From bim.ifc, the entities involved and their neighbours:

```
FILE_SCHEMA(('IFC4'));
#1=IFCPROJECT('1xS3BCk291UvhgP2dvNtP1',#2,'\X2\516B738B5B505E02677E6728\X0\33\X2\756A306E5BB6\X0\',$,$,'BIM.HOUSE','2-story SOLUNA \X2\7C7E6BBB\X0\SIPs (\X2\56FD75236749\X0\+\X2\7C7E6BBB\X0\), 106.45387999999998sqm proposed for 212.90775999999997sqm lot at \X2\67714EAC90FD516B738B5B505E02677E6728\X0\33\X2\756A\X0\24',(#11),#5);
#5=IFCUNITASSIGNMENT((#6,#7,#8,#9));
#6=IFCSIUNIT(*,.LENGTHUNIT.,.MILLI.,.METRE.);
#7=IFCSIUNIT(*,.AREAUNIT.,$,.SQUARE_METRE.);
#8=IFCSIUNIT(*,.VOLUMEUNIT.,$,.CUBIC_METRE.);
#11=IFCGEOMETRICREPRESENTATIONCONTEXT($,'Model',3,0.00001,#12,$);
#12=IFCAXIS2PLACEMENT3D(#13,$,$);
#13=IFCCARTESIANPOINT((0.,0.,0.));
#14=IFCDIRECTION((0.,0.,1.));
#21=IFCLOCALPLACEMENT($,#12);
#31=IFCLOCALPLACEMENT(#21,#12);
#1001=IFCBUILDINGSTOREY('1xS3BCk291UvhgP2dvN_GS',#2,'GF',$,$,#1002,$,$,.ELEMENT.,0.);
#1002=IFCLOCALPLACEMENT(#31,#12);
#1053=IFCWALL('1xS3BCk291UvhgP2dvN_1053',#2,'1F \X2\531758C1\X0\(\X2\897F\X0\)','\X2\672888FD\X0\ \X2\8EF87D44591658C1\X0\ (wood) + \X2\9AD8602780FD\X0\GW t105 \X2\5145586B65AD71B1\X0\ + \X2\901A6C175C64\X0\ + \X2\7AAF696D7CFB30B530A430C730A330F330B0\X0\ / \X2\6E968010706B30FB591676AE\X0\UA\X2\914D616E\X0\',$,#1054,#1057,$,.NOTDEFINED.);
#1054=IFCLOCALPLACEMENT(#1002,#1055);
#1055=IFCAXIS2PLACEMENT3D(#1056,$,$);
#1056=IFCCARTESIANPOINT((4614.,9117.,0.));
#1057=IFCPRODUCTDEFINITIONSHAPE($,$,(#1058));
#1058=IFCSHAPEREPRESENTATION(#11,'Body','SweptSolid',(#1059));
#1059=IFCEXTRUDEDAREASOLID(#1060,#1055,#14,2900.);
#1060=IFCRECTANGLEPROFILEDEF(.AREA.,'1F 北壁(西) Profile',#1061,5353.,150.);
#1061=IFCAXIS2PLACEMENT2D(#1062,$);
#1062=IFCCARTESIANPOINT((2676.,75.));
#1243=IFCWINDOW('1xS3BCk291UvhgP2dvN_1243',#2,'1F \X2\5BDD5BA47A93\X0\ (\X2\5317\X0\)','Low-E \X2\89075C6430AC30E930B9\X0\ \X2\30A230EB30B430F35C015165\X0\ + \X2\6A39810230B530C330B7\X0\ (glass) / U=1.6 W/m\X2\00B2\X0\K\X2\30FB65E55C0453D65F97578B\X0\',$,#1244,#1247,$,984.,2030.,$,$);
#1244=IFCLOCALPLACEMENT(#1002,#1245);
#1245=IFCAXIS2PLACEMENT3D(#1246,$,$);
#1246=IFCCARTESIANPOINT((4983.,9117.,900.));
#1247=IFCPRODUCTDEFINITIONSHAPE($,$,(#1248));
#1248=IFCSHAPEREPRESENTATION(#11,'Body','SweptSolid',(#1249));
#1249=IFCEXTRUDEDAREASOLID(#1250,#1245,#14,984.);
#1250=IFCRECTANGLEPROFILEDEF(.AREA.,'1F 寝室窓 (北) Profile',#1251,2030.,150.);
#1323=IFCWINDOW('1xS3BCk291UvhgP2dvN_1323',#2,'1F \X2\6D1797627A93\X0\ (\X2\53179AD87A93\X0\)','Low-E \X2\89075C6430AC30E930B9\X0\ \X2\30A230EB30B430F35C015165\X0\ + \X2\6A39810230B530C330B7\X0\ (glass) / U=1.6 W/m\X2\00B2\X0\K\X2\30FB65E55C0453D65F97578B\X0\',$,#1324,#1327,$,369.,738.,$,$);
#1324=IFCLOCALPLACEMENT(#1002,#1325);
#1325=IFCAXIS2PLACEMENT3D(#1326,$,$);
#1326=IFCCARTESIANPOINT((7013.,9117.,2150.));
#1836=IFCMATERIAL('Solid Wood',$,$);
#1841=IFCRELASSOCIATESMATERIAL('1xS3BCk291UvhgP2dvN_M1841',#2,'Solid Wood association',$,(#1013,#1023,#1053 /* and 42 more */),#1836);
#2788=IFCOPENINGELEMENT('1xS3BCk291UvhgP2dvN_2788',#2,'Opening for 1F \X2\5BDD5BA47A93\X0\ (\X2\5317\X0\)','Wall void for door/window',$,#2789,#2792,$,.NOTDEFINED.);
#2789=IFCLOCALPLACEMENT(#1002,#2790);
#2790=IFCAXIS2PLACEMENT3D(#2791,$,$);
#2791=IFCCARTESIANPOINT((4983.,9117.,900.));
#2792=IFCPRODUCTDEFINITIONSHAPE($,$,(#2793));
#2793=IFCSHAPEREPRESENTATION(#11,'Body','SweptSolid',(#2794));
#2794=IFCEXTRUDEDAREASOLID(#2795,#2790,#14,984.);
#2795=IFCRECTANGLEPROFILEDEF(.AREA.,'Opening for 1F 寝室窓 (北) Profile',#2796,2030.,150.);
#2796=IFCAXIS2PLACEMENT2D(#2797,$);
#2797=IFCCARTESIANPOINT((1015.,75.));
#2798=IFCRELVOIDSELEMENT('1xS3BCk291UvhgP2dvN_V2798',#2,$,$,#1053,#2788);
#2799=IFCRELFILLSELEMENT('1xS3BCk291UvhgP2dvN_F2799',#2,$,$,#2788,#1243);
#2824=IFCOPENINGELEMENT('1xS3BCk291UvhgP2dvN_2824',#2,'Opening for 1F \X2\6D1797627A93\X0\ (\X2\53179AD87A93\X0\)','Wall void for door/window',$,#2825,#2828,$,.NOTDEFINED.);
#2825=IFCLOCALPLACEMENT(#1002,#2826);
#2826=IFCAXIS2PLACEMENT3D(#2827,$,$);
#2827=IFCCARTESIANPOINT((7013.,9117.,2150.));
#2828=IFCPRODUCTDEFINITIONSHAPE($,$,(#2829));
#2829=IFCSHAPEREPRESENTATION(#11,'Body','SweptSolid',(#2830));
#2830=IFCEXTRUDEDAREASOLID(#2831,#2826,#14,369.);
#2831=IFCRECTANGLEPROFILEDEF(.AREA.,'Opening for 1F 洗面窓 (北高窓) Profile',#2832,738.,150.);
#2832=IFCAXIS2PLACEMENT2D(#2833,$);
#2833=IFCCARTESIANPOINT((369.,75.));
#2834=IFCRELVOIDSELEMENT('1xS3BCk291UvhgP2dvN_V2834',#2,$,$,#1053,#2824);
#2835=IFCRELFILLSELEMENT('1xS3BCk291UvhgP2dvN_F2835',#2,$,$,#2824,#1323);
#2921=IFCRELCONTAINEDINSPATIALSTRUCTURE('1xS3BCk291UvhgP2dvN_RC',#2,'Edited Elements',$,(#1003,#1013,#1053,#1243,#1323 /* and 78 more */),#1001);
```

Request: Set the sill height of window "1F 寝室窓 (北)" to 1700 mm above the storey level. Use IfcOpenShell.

```python
import numpy as np
import ifcopenshell
import ifcopenshell.api.geometry
import ifcopenshell.geom
import ifcopenshell.util.element
import ifcopenshell.util.placement
import ifcopenshell.util.shape
import ifcopenshell.util.unit

model = ifcopenshell.open("bim.ifc")
unit_scale = ifcopenshell.util.unit.calculate_unit_scale(model)

window = model.by_guid("1xS3BCk291UvhgP2dvN_1243")
opening = window.FillsVoids[0].RelatingOpeningElement
storey = ifcopenshell.util.element.get_container(window, ifc_class="IfcBuildingStorey")
level = ifcopenshell.util.placement.get_local_placement(storey.ObjectPlacement)[2, 3]

# The opening's origin need not be at the sill, so measure its lowest point.
shape = ifcopenshell.geom.create_shape(ifcopenshell.geom.settings(), opening)
bottom = ifcopenshell.util.shape.get_shape_bottom_elevation(shape, shape.geometry) / unit_scale
dz = level + 1.7 / unit_scale - bottom

shift = np.array([0.0, 0.0, dz])
# The window is not placed relative to its opening, so move both.
for product in (opening, window):
    matrix = ifcopenshell.util.placement.get_local_placement(product.ObjectPlacement)
    matrix[:3, 3] += shift
    ifcopenshell.api.geometry.edit_object_placement(model, product=product, matrix=matrix, is_si=False)

print(f"moved by {dz * unit_scale:+.3f} m")

model.write("bim-out.ifc")
```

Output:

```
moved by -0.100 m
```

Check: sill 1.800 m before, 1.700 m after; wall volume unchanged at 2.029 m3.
